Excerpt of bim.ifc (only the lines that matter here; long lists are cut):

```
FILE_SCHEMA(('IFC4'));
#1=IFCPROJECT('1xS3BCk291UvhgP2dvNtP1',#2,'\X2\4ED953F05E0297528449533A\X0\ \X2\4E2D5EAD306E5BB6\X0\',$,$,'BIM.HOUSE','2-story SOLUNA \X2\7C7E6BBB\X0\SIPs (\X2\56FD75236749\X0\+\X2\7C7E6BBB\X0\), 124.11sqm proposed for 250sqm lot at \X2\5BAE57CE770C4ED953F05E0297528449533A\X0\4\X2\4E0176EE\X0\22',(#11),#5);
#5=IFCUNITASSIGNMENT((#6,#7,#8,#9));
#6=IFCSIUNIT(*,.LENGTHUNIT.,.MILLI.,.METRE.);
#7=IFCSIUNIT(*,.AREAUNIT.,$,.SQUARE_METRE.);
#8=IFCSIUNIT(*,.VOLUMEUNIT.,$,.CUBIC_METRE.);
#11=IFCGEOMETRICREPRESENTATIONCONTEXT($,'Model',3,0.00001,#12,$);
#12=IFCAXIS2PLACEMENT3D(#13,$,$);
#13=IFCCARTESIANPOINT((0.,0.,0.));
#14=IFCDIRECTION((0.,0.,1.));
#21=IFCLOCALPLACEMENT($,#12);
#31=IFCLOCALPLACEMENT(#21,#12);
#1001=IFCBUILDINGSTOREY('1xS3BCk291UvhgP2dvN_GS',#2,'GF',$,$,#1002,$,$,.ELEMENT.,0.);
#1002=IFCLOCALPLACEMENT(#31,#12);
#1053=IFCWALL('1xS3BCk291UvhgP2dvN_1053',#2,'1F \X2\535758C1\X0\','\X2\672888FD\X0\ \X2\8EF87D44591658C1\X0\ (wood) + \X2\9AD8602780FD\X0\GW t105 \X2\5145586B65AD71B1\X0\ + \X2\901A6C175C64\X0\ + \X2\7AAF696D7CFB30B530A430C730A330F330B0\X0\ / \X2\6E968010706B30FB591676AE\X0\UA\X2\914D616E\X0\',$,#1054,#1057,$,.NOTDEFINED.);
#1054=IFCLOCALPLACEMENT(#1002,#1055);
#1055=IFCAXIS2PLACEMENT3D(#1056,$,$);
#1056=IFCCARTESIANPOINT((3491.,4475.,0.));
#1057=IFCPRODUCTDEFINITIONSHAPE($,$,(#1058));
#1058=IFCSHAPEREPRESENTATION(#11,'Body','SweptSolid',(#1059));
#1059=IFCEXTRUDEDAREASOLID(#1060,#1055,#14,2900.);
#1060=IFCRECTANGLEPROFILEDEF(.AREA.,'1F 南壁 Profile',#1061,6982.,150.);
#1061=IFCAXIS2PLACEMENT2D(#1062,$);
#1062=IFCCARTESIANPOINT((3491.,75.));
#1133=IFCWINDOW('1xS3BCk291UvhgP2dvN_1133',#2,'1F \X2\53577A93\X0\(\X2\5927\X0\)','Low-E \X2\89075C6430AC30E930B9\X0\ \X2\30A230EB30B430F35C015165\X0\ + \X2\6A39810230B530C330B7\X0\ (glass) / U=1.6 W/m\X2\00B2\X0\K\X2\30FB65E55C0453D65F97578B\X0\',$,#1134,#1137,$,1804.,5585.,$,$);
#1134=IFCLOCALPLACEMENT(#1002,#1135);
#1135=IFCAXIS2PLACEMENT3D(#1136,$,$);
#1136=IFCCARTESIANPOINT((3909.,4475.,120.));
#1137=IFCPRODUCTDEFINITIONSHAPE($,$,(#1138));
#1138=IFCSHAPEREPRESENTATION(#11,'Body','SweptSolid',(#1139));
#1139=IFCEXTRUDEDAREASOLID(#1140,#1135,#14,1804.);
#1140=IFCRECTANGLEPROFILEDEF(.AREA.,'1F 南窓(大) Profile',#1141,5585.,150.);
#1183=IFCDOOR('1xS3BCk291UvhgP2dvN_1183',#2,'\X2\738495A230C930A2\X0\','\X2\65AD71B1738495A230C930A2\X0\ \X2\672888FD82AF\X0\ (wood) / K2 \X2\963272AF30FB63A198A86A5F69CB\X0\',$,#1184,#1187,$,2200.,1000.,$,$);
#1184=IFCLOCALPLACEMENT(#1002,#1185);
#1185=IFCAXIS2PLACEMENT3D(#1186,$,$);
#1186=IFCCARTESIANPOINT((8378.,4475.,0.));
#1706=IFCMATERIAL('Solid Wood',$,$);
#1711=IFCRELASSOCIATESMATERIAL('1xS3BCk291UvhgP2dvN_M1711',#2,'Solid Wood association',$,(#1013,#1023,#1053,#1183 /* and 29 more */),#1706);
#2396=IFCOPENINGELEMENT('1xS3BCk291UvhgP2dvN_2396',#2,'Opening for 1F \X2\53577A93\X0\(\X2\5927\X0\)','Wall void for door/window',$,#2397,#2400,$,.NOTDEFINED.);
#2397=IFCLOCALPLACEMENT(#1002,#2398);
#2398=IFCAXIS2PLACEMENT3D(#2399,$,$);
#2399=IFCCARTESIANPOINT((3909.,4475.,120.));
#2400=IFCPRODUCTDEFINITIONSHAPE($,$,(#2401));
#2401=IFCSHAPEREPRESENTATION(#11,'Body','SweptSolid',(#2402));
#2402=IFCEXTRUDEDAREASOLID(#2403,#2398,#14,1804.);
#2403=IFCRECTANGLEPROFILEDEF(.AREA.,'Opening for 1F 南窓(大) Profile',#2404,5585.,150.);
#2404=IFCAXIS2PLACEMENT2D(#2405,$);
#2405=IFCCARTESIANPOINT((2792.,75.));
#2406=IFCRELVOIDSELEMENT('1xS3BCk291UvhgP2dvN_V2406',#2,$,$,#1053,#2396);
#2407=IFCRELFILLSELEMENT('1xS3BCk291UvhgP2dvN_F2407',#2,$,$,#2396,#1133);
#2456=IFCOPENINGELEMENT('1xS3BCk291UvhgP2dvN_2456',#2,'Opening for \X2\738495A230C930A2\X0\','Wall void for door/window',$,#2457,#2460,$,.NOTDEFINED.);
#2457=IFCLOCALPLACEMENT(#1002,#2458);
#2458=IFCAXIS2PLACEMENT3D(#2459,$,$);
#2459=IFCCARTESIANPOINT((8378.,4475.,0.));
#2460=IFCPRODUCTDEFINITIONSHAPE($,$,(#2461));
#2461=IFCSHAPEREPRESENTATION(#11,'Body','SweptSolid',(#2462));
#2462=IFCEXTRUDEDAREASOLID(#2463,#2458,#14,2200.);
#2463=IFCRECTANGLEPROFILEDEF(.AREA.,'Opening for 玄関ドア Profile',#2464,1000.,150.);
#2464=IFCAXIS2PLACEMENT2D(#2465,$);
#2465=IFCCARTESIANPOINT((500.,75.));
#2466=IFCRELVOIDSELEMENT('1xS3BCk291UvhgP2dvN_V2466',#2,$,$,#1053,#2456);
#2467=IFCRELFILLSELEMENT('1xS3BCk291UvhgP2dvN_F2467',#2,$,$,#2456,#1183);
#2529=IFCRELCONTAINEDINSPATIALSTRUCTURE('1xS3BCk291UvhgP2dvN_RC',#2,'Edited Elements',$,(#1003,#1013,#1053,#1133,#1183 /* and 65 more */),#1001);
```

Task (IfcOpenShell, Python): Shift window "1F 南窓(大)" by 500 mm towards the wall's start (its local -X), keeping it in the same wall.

```python
import ifcopenshell
import ifcopenshell.api.geometry
import ifcopenshell.util.placement
import ifcopenshell.util.unit

model = ifcopenshell.open("bim.ifc")
unit_scale = ifcopenshell.util.unit.calculate_unit_scale(model)

window = model.by_id(1133)
opening = window.FillsVoids[0].RelatingOpeningElement
wall = opening.VoidsElements[0].RelatingBuildingElement

wall_matrix = ifcopenshell.util.placement.get_local_placement(wall.ObjectPlacement)
shift = wall_matrix[:3, 0] * -0.5 / unit_scale
before = ifcopenshell.util.placement.get_local_placement(window.ObjectPlacement)[:3, 3].copy()

# The window is not placed relative to its opening, so move both.
for product in (opening, window):
    matrix = ifcopenshell.util.placement.get_local_placement(product.ObjectPlacement)
    matrix[:3, 3] += shift
    ifcopenshell.api.geometry.edit_object_placement(model, product=product, matrix=matrix, is_si=False)

after = ifcopenshell.util.placement.get_local_placement(window.ObjectPlacement)[:3, 3]
print("window moved by", (after - before).round(3) + 0.0)

model.write("bim_rev.ifc")
```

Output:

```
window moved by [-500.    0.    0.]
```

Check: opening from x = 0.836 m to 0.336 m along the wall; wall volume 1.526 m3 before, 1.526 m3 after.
